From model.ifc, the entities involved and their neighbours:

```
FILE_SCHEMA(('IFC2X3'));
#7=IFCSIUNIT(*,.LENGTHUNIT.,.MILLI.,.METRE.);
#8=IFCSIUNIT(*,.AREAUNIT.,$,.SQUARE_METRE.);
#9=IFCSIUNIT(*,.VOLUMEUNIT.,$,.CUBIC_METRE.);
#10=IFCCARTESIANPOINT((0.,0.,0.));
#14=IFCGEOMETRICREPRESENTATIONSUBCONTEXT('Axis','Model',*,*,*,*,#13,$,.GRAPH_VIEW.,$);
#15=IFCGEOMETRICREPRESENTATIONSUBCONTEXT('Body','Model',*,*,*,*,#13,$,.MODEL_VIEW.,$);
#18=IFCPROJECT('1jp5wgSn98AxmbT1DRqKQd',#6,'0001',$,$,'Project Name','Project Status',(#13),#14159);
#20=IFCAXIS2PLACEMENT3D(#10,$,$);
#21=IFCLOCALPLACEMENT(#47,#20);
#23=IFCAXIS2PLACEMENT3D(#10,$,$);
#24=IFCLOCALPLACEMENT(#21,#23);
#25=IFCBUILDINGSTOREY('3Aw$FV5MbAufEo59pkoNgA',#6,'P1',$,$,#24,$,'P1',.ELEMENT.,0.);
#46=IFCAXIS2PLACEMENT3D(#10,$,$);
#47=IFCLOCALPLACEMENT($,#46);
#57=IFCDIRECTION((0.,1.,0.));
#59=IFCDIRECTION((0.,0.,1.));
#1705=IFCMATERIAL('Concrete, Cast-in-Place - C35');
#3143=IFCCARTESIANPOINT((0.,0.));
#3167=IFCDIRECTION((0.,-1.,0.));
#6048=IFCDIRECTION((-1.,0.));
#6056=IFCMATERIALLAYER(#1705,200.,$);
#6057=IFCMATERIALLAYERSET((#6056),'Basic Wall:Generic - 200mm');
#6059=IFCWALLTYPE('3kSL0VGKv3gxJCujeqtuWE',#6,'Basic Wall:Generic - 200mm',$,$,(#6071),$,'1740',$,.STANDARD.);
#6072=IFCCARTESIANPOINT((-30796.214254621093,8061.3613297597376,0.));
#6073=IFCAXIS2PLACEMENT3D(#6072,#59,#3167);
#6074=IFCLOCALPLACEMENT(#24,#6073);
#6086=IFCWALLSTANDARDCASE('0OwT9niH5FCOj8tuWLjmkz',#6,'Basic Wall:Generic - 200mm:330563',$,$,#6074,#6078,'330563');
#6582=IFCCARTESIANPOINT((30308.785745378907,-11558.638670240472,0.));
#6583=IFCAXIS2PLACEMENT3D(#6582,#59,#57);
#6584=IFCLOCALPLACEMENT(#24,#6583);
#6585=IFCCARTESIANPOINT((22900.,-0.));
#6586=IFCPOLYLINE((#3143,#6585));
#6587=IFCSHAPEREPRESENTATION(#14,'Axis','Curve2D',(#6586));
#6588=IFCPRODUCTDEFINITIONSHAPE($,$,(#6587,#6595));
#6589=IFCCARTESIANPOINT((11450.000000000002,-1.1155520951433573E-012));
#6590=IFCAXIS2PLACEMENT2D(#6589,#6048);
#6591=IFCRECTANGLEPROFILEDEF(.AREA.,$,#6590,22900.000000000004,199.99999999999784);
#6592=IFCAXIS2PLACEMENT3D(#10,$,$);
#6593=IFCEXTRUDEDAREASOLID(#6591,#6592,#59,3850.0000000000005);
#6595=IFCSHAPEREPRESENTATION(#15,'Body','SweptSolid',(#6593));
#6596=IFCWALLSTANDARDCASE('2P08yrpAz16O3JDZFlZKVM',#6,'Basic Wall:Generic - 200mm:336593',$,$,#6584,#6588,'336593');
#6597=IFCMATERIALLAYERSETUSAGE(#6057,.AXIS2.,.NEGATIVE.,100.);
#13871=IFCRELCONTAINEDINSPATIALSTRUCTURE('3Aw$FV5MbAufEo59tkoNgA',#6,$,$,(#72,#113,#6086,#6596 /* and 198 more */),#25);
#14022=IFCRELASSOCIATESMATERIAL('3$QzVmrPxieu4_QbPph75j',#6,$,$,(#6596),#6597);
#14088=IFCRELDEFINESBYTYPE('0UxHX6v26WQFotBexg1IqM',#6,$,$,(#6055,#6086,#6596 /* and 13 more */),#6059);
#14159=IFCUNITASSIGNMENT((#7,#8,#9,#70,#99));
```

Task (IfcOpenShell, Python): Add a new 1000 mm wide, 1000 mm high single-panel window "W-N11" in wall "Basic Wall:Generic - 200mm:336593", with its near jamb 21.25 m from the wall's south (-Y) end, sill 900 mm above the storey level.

```python
import numpy as np
import ifcopenshell
import ifcopenshell.api.feature
import ifcopenshell.api.geometry
import ifcopenshell.api.root
import ifcopenshell.api.spatial
import ifcopenshell.api.type
import ifcopenshell.geom
import ifcopenshell.util.element
import ifcopenshell.util.placement
import ifcopenshell.util.representation
import ifcopenshell.util.shape
import ifcopenshell.util.unit

model = ifcopenshell.open("model.ifc")
unit_scale = ifcopenshell.util.unit.calculate_unit_scale(model)
settings = ifcopenshell.geom.settings()


def volume(element):
    """Net volume in cubic metres, openings subtracted."""
    shape = ifcopenshell.geom.create_shape(settings, element)
    return ifcopenshell.util.shape.get_volume(shape.geometry)


wall = model.by_id(6596)
storey = ifcopenshell.util.element.get_container(wall, ifc_class="IfcBuildingStorey")
context = ifcopenshell.util.representation.get_context(model, "Model", "Body", "MODEL_VIEW")
before = volume(wall)

width, height, from_end, sill = 1, 1, 21.25, 0.9  # metres

# The wall runs along its own X axis, and the end named is its -X end.
wall_shape = ifcopenshell.geom.create_shape(settings, wall)
x, y, z = ifcopenshell.util.shape.get_vertices(wall_shape.geometry).T
start = x.min() + from_end
face, thickness = float(y.min()), float(y.max() - y.min())
wall_matrix = ifcopenshell.util.placement.get_local_placement(wall.ObjectPlacement)
level = ifcopenshell.util.placement.get_local_placement(storey.ObjectPlacement)[2, 3]


def in_wall(x, y):
    """Placement at x, y metres in the wall's axes, at sill height."""
    matrix = wall_matrix.copy()
    matrix[:, 3] = wall_matrix @ np.array([x / unit_scale, y / unit_scale, 0.0, 1.0])
    matrix[2, 3] = level + sill / unit_scale
    return matrix


# Opening: a box that overshoots both wall faces by 50 mm.
opening = ifcopenshell.api.root.create_entity(model, ifc_class="IfcOpeningElement")
box = ifcopenshell.api.geometry.add_wall_representation(
    model, context=context, length=width, height=height, thickness=thickness + 0.1
)
ifcopenshell.api.geometry.assign_representation(model, product=opening, representation=box)
ifcopenshell.api.geometry.edit_object_placement(model, product=opening, matrix=in_wall(start, face - 0.05), is_si=False)
ifcopenshell.api.feature.add_feature(model, feature=opening, element=wall)

window = ifcopenshell.api.root.create_entity(model, ifc_class="IfcWindow", name="W-N11")
window.OverallWidth, window.OverallHeight = width / unit_scale, height / unit_scale
body = ifcopenshell.api.geometry.add_window_representation(
    model,
    context=context,
    overall_width=window.OverallWidth,
    overall_height=window.OverallHeight,
    partition_type="SINGLE_PANEL",
)
ifcopenshell.api.geometry.assign_representation(model, product=window, representation=body)
ifcopenshell.api.spatial.assign_container(model, products=[window], relating_structure=storey)
fills = ifcopenshell.api.feature.add_filling(model, opening=opening, element=window)
fills.OwnerHistory = window.OwnerHistory  # required in IFC2X3

# IFC2X3 keeps the operation on the window style.
style = ifcopenshell.api.root.create_entity(model, ifc_class="IfcWindowStyle", name="W-N11")
style.OperationType, style.ConstructionType = "SINGLE_PANEL", "NOTDEFINED"
style.ParameterTakesPrecedence = style.Sizeable = False
ifcopenshell.api.type.assign_type(model, related_objects=[window], relating_type=style)

# Centre the window in the wall's thickness.
ifcopenshell.api.geometry.edit_object_placement(model, product=window, matrix=in_wall(start, face), is_si=False)
window_shape = ifcopenshell.geom.create_shape(settings, window)
depth = ifcopenshell.util.shape.get_vertices(window_shape.geometry)[:, 1]
offset = face + thickness / 2 - (depth.min() + depth.max()) / 2
ifcopenshell.api.geometry.edit_object_placement(model, product=window, matrix=in_wall(start, offset), is_si=False)

after = volume(wall)

print(f"wall volume {before:.3f} -> {after:.3f} m3")

model.write("model_updated.ifc")
```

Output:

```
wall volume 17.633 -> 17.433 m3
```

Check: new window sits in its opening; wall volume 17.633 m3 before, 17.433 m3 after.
